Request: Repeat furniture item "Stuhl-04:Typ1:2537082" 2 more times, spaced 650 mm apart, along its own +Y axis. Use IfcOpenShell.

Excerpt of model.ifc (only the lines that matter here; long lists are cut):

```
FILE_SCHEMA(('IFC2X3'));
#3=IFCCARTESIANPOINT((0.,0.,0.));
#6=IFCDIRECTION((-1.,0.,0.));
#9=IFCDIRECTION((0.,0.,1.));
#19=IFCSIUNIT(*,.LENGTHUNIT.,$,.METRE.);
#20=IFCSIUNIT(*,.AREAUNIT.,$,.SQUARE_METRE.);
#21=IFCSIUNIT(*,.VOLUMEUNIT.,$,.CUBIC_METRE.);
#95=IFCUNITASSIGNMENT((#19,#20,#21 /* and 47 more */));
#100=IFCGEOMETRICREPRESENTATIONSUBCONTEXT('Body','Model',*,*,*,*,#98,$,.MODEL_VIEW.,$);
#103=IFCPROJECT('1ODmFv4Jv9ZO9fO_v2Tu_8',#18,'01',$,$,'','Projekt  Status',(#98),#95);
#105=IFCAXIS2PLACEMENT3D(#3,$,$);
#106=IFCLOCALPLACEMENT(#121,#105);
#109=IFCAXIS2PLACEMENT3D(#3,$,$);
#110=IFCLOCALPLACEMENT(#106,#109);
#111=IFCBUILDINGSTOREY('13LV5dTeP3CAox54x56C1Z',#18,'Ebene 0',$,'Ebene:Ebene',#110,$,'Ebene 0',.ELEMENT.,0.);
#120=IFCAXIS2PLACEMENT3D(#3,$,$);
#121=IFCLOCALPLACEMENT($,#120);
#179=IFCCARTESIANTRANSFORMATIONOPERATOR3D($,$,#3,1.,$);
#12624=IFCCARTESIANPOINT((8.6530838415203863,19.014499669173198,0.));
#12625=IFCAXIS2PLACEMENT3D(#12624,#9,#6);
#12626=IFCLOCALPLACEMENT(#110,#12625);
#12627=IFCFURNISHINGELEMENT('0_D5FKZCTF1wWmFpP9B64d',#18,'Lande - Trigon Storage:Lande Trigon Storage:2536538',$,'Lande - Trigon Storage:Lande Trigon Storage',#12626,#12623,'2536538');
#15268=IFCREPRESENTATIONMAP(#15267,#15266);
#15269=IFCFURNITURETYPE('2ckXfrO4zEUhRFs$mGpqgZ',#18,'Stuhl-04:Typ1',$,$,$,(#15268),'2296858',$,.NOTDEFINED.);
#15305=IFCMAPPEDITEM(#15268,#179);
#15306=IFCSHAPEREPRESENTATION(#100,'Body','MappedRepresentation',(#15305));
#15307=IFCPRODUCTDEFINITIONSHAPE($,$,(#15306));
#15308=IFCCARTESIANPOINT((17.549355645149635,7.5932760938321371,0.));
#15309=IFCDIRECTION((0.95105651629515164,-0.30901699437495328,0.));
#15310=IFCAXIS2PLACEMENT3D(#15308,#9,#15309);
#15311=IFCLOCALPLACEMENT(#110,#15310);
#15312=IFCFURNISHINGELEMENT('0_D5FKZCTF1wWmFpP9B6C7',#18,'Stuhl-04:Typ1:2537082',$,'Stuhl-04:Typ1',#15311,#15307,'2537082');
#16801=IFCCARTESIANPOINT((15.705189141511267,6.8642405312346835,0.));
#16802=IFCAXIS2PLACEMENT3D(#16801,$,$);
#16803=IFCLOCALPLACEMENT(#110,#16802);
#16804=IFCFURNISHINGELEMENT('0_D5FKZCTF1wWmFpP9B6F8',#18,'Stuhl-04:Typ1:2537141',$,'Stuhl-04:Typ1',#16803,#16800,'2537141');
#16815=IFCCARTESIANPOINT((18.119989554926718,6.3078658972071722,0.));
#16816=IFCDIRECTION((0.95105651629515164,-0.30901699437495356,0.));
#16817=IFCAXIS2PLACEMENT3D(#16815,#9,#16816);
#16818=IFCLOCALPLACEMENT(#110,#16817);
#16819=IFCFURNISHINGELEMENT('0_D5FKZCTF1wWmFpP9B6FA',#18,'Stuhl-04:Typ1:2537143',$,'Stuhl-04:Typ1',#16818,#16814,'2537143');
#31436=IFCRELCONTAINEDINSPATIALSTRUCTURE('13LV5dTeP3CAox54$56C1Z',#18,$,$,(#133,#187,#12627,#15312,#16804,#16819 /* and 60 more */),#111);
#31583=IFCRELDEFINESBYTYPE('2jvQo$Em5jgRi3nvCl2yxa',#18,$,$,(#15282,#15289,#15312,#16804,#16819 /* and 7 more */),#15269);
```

```python
import ifcopenshell
import ifcopenshell.api.geometry
import ifcopenshell.api.root
import ifcopenshell.util.element
import ifcopenshell.util.placement

model = ifcopenshell.open("model.ifc")

source = model.by_guid("0_D5FKZCTF1wWmFpP9B6C7")
base = ifcopenshell.util.placement.get_local_placement(source.ObjectPlacement)
step = base[:3, 1] * 0.65

for i in range(1, 3):
    copy = ifcopenshell.api.root.copy_class(model, product=source)
    copy.Representation = ifcopenshell.util.element.copy_deep(
        model, source.Representation, exclude=["IfcGeometricRepresentationContext", "IfcRepresentationMap"]
    )
    copy.Name = "Stuhl-04:Typ1"
    copy.Tag = None
    matrix = base.copy()
    matrix[:3, 3] += i * step
    print("added at", matrix[:3, 3].round(3) + 0.0)
    ifcopenshell.api.geometry.edit_object_placement(model, product=copy, matrix=matrix, is_si=False)

model.write("model-out.ifc")
```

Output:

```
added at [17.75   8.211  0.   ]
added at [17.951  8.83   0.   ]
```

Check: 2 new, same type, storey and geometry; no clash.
